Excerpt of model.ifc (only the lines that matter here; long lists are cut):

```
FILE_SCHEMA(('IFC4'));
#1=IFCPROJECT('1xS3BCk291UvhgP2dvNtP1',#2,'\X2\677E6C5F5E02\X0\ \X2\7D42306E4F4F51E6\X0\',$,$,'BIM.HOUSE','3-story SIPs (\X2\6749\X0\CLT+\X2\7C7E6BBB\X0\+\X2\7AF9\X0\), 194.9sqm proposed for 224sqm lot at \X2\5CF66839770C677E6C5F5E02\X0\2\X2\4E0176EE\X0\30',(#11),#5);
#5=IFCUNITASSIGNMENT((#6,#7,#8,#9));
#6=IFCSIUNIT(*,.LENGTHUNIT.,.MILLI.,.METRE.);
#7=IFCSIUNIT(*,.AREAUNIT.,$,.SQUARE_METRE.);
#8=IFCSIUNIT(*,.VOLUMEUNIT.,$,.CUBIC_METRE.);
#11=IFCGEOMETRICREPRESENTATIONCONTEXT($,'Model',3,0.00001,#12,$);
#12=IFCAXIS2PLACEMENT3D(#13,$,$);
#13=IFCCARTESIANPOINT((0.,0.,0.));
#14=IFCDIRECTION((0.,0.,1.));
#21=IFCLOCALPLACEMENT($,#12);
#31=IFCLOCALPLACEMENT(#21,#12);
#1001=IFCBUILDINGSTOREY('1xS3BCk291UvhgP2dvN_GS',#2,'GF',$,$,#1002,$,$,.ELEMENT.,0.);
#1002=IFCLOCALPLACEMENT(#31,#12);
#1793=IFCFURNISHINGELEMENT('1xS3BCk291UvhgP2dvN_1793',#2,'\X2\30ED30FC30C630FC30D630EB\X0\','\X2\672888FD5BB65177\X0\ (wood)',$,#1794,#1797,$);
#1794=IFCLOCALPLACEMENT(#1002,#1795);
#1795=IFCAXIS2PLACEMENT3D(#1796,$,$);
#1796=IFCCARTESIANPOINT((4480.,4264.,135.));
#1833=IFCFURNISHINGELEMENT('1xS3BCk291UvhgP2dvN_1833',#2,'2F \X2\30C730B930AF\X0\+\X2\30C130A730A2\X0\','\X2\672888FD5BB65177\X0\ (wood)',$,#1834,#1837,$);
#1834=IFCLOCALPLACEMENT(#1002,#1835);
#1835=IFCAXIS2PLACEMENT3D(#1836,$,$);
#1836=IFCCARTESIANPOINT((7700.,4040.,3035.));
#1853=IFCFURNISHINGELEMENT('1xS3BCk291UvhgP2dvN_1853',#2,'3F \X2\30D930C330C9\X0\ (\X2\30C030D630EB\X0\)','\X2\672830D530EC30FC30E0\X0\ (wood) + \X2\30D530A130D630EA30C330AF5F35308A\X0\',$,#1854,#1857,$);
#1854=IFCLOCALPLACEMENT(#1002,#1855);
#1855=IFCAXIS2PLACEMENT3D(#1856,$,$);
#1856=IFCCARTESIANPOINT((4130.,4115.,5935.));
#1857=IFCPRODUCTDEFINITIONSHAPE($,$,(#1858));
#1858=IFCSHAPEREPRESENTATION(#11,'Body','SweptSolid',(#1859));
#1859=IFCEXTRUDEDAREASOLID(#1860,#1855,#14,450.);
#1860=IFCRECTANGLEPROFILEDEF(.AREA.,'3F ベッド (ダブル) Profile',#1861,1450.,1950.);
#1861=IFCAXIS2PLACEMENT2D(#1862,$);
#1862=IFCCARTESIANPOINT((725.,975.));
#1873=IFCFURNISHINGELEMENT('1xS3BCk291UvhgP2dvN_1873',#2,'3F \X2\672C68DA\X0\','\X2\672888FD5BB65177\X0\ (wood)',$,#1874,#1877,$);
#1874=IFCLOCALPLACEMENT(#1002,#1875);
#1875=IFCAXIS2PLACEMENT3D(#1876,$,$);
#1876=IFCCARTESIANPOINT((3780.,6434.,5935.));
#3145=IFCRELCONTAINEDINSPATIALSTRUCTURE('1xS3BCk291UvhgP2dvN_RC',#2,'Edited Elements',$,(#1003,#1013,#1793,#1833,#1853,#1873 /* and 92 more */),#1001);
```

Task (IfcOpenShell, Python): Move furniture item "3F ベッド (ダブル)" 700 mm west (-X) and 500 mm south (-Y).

```python
import ifcopenshell
import ifcopenshell.api.geometry
import ifcopenshell.util.placement
import ifcopenshell.util.unit

model = ifcopenshell.open("model.ifc")
unit_scale = ifcopenshell.util.unit.calculate_unit_scale(model)

item = model.by_guid("1xS3BCk291UvhgP2dvN_1853")
matrix = ifcopenshell.util.placement.get_local_placement(item.ObjectPlacement)
matrix[0, 3] -= 0.7 / unit_scale
matrix[1, 3] -= 0.5 / unit_scale
ifcopenshell.api.geometry.edit_object_placement(model, product=item, matrix=matrix, is_si=False)

print(ifcopenshell.util.placement.get_local_placement(item.ObjectPlacement).round(3) + 0.0)

model.write("model_edited.ifc")
```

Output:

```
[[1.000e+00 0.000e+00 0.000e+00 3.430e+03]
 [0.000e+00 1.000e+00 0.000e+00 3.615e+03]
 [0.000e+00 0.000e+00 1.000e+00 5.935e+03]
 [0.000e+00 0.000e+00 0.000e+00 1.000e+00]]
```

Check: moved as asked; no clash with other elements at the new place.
